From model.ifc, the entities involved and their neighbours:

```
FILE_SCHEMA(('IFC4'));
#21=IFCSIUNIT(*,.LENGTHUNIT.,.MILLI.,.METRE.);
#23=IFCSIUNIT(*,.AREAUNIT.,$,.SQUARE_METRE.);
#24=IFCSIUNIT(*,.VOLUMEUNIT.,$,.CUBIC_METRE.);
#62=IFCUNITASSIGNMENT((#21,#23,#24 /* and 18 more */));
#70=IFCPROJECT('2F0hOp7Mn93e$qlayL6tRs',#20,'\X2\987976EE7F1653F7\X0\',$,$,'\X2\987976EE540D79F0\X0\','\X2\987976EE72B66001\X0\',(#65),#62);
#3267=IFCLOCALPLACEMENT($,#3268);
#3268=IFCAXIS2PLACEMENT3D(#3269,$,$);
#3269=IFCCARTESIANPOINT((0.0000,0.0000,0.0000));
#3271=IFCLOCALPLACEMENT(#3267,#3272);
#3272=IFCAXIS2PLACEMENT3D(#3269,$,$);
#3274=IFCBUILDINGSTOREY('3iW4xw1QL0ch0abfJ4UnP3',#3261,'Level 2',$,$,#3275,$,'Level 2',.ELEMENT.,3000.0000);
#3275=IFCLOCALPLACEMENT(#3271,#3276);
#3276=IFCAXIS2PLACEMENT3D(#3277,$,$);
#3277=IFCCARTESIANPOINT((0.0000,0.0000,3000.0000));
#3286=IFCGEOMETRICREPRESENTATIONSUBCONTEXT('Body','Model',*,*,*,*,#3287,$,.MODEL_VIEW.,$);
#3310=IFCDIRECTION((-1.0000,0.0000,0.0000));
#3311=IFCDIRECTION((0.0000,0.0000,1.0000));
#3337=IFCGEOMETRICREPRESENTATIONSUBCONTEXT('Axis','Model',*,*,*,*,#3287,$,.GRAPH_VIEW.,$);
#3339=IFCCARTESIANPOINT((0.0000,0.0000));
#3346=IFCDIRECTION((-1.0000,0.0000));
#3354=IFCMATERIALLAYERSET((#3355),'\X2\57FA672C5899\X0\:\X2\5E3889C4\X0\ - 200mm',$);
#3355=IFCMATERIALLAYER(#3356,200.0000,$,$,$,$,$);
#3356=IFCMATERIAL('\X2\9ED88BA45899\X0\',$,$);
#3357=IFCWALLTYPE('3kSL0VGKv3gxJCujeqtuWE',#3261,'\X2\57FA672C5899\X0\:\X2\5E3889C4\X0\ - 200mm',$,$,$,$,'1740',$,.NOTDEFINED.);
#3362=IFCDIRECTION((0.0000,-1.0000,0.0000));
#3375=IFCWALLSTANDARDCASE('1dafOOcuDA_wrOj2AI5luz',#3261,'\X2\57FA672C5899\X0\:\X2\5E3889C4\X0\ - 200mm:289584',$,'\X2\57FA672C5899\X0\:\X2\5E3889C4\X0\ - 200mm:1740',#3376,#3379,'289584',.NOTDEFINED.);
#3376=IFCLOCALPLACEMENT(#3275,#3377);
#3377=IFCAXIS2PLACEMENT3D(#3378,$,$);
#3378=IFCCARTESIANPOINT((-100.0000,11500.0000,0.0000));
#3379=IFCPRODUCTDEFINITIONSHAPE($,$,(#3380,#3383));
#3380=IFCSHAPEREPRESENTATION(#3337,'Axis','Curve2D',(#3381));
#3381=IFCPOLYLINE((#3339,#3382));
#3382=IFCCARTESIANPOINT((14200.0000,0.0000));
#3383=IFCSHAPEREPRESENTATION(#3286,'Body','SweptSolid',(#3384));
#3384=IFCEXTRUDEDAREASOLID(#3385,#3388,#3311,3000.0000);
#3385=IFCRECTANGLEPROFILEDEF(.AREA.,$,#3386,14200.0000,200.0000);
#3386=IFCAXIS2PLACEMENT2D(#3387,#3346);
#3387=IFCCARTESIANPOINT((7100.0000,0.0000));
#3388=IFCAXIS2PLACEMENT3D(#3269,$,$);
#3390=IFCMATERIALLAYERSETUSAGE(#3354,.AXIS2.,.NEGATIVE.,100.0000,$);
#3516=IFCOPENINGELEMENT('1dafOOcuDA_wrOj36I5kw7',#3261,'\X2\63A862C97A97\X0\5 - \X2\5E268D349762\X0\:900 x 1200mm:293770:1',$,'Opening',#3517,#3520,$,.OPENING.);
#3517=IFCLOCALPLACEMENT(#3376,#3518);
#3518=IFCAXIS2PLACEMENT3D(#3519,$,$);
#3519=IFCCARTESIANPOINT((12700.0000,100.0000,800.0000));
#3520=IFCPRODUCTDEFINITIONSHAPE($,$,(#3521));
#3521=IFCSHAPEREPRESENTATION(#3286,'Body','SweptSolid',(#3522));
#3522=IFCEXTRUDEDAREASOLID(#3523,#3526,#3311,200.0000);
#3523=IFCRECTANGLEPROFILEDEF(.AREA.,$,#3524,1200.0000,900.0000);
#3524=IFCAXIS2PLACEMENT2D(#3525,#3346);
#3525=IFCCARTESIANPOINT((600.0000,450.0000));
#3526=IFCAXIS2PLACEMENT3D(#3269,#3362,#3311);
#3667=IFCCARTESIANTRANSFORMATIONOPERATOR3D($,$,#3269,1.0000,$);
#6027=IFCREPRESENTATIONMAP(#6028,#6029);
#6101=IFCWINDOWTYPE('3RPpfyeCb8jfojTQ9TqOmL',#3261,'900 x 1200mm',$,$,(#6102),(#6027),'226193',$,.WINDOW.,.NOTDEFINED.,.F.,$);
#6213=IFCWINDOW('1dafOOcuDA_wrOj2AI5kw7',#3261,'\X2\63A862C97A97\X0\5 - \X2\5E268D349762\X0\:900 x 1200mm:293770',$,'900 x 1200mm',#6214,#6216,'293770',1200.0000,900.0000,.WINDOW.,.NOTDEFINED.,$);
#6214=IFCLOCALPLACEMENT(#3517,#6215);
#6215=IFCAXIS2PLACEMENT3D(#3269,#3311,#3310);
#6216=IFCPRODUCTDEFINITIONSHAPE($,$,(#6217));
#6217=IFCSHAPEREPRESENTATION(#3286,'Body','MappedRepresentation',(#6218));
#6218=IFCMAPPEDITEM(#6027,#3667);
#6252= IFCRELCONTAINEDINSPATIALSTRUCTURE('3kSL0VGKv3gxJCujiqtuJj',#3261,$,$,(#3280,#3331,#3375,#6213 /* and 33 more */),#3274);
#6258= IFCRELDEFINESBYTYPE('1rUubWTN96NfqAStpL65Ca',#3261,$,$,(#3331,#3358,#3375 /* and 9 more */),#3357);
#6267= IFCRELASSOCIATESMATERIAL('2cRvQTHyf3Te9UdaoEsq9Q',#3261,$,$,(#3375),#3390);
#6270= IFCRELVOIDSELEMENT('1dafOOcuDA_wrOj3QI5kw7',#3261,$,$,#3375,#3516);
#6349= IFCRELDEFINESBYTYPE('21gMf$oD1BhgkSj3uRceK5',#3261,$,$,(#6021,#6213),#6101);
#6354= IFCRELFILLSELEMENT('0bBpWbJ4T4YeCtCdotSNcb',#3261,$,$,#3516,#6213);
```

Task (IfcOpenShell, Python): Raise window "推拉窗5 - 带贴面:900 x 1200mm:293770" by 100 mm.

```python
import numpy as np
import ifcopenshell
import ifcopenshell.api.geometry
import ifcopenshell.util.placement
import ifcopenshell.util.unit

model = ifcopenshell.open("model.ifc")
unit_scale = ifcopenshell.util.unit.calculate_unit_scale(model)

window = model.by_id(6213)
opening = window.FillsVoids[0].RelatingOpeningElement
dz = 100.0

shift = np.array([0.0, 0.0, dz])
# The window is placed relative to its opening, so it follows when the opening moves.
matrix = ifcopenshell.util.placement.get_local_placement(opening.ObjectPlacement)
matrix[:3, 3] += shift
ifcopenshell.api.geometry.edit_object_placement(
    model, product=opening, matrix=matrix, is_si=False, should_transform_children=True
)

print(f"moved by {dz * unit_scale:+.3f} m")

model.write("model_v2.ifc")
```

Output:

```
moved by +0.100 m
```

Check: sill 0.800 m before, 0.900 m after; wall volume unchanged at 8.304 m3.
